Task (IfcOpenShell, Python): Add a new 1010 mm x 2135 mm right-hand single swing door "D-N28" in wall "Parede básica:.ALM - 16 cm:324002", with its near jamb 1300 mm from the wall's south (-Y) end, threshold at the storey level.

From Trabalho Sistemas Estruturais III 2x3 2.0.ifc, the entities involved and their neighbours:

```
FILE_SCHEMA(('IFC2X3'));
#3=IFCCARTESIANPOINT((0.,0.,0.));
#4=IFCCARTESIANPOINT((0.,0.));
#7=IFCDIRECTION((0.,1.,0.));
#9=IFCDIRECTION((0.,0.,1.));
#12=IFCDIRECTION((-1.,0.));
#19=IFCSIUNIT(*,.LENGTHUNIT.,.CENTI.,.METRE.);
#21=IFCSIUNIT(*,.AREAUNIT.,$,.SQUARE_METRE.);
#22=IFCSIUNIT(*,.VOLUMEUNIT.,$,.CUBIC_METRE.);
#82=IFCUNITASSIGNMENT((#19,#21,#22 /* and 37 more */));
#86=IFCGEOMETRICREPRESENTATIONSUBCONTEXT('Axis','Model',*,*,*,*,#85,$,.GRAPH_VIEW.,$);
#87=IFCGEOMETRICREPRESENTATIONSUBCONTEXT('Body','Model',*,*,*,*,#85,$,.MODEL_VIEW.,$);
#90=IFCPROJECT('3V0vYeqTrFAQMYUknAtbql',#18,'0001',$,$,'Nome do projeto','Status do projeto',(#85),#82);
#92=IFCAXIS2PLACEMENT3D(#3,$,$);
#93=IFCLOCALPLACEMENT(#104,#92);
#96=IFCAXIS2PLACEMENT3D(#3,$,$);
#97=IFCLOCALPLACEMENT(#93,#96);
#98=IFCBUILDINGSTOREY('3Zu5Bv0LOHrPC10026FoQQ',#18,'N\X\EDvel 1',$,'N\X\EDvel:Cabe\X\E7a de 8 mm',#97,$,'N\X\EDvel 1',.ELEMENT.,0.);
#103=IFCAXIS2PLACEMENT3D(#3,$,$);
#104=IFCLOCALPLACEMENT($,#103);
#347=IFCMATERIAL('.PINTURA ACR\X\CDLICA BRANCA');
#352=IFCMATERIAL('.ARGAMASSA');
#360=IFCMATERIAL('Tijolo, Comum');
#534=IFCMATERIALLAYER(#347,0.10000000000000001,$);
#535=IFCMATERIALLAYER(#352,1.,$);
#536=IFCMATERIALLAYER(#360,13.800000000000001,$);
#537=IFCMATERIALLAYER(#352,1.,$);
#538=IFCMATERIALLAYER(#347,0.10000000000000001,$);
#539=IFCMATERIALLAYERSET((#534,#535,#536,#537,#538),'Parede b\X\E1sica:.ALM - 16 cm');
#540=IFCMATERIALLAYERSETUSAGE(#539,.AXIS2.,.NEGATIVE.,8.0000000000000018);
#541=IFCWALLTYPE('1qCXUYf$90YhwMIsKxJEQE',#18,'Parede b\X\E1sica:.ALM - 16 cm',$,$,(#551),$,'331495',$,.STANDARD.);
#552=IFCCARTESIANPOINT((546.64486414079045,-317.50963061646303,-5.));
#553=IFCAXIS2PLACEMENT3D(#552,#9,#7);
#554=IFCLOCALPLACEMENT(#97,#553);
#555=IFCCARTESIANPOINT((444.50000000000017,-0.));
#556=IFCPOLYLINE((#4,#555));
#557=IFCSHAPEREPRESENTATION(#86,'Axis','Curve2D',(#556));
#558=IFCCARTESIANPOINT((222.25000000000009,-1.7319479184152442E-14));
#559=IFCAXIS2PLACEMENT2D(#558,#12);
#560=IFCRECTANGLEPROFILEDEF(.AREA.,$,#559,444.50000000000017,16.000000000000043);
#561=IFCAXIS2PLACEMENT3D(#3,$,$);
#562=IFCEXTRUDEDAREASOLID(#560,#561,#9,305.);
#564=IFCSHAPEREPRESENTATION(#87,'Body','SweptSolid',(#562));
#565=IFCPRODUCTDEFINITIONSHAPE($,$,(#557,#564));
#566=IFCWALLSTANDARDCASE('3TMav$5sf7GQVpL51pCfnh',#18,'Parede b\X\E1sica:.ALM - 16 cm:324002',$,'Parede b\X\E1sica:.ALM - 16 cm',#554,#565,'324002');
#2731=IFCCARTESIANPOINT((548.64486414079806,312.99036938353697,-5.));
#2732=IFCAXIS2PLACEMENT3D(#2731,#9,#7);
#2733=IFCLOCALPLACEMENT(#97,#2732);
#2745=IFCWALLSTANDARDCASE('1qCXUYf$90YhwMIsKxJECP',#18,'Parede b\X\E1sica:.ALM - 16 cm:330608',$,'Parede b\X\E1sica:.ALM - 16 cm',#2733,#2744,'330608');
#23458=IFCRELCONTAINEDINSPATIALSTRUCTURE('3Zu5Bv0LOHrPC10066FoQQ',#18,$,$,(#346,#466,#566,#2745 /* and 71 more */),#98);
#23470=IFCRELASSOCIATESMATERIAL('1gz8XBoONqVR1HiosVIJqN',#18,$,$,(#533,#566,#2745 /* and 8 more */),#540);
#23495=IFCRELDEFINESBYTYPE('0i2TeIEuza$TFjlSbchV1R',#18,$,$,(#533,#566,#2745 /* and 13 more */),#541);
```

```python
import numpy as np
import ifcopenshell
import ifcopenshell.api.feature
import ifcopenshell.api.geometry
import ifcopenshell.api.root
import ifcopenshell.api.spatial
import ifcopenshell.api.type
import ifcopenshell.geom
import ifcopenshell.util.element
import ifcopenshell.util.placement
import ifcopenshell.util.representation
import ifcopenshell.util.shape
import ifcopenshell.util.unit

model = ifcopenshell.open("Trabalho Sistemas Estruturais III 2x3 2.0.ifc")
unit_scale = ifcopenshell.util.unit.calculate_unit_scale(model)
settings = ifcopenshell.geom.settings()


def volume(element):
    """Net volume in cubic metres, openings subtracted."""
    shape = ifcopenshell.geom.create_shape(settings, element)
    return ifcopenshell.util.shape.get_volume(shape.geometry)


wall = model.by_id(566)
storey = ifcopenshell.util.element.get_container(wall, ifc_class="IfcBuildingStorey")
context = ifcopenshell.util.representation.get_context(model, "Model", "Body", "MODEL_VIEW")
before = volume(wall)

width, height, from_end, sill = 1.01, 2.135, 1.3, 0.0  # metres

# The wall runs along its own X axis, and the end named is its -X end.
wall_shape = ifcopenshell.geom.create_shape(settings, wall)
x, y, z = ifcopenshell.util.shape.get_vertices(wall_shape.geometry).T
start = x.min() + from_end
face, thickness = float(y.min()), float(y.max() - y.min())
wall_matrix = ifcopenshell.util.placement.get_local_placement(wall.ObjectPlacement)
level = ifcopenshell.util.placement.get_local_placement(storey.ObjectPlacement)[2, 3]


def in_wall(x, y):
    """Placement at x, y metres in the wall's axes, at sill height."""
    matrix = wall_matrix.copy()
    matrix[:, 3] = wall_matrix @ np.array([x / unit_scale, y / unit_scale, 0.0, 1.0])
    matrix[2, 3] = level + sill / unit_scale
    return matrix


# Opening: a box that overshoots both wall faces by 50 mm.
opening = ifcopenshell.api.root.create_entity(model, ifc_class="IfcOpeningElement")
box = ifcopenshell.api.geometry.add_wall_representation(
    model, context=context, length=width, height=height, thickness=thickness + 0.1
)
ifcopenshell.api.geometry.assign_representation(model, product=opening, representation=box)
ifcopenshell.api.geometry.edit_object_placement(model, product=opening, matrix=in_wall(start, face - 0.05), is_si=False)
ifcopenshell.api.feature.add_feature(model, feature=opening, element=wall)

door = ifcopenshell.api.root.create_entity(model, ifc_class="IfcDoor", name="D-N28")
door.OverallWidth, door.OverallHeight = width / unit_scale, height / unit_scale
body = ifcopenshell.api.geometry.add_door_representation(
    model,
    context=context,
    overall_width=door.OverallWidth,
    overall_height=door.OverallHeight,
    operation_type="SINGLE_SWING_RIGHT",
    lining_properties={"LiningDepth": thickness / unit_scale, "ThresholdDepth": thickness / unit_scale},
)
ifcopenshell.api.geometry.assign_representation(model, product=door, representation=body)
ifcopenshell.api.spatial.assign_container(model, products=[door], relating_structure=storey)
fills = ifcopenshell.api.feature.add_filling(model, opening=opening, element=door)
fills.OwnerHistory = door.OwnerHistory  # required in IFC2X3

# IFC2X3 keeps the operation on the door style.
style = ifcopenshell.api.root.create_entity(model, ifc_class="IfcDoorStyle", name="D-N28")
style.OperationType, style.ConstructionType = "SINGLE_SWING_RIGHT", "NOTDEFINED"
style.ParameterTakesPrecedence = style.Sizeable = False
ifcopenshell.api.type.assign_type(model, related_objects=[door], relating_type=style)

# The lining spans the wall, so the door starts at the wall face.
ifcopenshell.api.geometry.edit_object_placement(model, product=door, matrix=in_wall(start, face), is_si=False)

after = volume(wall)

print(f"wall volume {before:.3f} -> {after:.3f} m3")

model.write("Trabalho Sistemas Estruturais III 2x3 2.0_rev.ifc")
```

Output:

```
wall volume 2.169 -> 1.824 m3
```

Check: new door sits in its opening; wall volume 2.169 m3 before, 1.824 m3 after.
